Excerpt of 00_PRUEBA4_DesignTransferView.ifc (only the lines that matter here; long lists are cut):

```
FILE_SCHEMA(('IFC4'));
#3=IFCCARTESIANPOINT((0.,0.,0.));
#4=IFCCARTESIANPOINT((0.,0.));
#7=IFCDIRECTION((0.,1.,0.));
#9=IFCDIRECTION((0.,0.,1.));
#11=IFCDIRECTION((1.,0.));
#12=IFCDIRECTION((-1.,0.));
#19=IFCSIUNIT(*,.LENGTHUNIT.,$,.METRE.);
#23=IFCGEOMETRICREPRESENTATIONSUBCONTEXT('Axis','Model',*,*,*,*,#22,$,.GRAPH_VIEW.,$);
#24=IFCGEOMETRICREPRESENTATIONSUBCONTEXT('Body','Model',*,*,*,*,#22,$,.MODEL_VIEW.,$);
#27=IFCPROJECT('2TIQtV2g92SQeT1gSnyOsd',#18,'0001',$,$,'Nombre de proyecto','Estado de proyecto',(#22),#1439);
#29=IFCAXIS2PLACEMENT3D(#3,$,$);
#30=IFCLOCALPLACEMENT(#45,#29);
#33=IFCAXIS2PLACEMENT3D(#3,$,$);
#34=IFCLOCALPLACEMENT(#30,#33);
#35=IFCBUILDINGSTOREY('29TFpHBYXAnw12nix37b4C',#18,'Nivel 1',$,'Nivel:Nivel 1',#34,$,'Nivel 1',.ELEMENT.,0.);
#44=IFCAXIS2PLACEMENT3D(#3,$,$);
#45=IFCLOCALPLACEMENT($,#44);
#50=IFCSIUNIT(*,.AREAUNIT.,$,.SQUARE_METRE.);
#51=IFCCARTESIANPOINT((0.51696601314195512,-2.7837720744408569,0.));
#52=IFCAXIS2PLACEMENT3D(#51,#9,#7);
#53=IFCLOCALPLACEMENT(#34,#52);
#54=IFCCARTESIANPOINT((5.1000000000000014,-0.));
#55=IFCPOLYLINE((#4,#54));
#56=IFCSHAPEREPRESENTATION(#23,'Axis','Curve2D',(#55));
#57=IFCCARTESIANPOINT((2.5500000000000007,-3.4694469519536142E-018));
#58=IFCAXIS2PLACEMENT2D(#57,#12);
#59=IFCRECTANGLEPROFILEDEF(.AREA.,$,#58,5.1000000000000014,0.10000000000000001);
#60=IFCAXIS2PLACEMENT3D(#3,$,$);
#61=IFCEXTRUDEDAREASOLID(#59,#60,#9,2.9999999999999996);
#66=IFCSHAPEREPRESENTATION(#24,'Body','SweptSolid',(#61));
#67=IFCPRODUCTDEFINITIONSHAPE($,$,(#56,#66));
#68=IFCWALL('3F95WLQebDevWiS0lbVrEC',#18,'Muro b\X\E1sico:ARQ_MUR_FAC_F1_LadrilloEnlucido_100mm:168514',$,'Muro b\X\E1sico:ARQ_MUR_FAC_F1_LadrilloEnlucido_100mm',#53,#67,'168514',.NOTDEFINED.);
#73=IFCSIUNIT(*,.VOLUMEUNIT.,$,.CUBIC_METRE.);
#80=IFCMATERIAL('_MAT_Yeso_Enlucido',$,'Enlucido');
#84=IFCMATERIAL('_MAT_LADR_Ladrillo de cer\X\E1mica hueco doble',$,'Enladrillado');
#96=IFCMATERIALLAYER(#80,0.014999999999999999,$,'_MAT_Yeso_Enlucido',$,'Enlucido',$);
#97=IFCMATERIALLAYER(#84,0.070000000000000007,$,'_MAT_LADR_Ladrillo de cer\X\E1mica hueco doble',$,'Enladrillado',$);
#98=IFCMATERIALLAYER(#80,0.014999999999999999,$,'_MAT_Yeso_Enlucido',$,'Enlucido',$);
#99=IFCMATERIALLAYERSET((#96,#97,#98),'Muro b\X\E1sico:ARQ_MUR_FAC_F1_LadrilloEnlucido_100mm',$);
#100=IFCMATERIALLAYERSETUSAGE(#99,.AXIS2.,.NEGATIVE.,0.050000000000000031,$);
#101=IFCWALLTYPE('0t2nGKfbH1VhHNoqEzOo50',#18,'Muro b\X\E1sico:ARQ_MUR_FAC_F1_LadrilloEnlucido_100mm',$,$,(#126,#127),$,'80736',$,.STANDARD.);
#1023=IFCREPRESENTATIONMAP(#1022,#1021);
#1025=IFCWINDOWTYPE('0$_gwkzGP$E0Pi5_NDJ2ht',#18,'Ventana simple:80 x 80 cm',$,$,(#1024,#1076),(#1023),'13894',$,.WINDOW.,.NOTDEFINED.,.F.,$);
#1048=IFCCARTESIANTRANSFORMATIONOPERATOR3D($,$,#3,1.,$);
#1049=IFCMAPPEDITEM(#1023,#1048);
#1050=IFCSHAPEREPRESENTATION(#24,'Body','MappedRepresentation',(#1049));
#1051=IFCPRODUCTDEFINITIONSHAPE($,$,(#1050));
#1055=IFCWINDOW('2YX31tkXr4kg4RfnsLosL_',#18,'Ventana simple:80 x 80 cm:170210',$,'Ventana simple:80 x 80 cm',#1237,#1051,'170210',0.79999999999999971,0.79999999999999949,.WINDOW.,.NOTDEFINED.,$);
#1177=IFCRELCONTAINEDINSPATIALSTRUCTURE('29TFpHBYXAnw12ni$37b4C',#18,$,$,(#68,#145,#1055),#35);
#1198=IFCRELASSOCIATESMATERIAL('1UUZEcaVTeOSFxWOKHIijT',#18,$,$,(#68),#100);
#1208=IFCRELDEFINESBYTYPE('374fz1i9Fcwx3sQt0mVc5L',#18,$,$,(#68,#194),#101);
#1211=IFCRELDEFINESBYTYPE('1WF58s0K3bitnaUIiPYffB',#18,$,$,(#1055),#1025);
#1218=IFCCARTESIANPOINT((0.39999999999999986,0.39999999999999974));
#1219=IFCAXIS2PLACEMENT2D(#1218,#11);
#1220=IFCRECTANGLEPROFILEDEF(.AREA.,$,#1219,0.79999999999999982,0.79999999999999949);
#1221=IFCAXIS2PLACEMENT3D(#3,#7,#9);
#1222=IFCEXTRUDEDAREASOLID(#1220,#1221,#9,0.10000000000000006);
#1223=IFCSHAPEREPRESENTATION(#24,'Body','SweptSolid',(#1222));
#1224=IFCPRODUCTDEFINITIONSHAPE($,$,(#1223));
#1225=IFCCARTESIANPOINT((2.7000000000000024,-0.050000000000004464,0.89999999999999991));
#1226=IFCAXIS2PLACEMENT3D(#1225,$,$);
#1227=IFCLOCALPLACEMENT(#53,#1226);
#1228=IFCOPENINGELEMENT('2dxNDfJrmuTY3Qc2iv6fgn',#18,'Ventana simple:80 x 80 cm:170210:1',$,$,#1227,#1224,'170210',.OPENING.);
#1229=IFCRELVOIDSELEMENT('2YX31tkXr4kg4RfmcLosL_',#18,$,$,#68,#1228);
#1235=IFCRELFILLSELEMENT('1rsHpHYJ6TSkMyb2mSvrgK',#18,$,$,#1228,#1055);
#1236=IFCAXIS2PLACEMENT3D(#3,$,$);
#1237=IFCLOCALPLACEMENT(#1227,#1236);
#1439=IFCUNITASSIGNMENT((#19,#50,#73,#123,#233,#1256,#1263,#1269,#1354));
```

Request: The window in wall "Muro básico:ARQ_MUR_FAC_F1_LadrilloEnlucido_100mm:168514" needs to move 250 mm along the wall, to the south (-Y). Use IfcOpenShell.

```python
import ifcopenshell
import ifcopenshell.api.geometry
import ifcopenshell.util.placement
import ifcopenshell.util.unit

model = ifcopenshell.open("00_PRUEBA4_DesignTransferView.ifc")
unit_scale = ifcopenshell.util.unit.calculate_unit_scale(model)

window = model.by_guid("2YX31tkXr4kg4RfnsLosL_")
opening = window.FillsVoids[0].RelatingOpeningElement
wall = opening.VoidsElements[0].RelatingBuildingElement

wall_matrix = ifcopenshell.util.placement.get_local_placement(wall.ObjectPlacement)
shift = wall_matrix[:3, 0] * -0.25 / unit_scale
before = ifcopenshell.util.placement.get_local_placement(window.ObjectPlacement)[:3, 3].copy()

# The window is placed relative to its opening, so it follows when the opening moves.
matrix = ifcopenshell.util.placement.get_local_placement(opening.ObjectPlacement)
matrix[:3, 3] += shift
ifcopenshell.api.geometry.edit_object_placement(
    model, product=opening, matrix=matrix, is_si=False, should_transform_children=True
)

after = ifcopenshell.util.placement.get_local_placement(window.ObjectPlacement)[:3, 3]
print("window moved by", (after - before).round(3) + 0.0)

model.write("00_PRUEBA4_DesignTransferView_edited.ifc")
```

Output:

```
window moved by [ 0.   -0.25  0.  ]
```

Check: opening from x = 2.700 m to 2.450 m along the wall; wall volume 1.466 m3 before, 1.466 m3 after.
